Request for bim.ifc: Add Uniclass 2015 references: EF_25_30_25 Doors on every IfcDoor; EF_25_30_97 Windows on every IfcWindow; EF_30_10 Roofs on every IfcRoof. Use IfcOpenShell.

First a look at what the model holds.

```python
import ifcopenshell

model = ifcopenshell.open("bim.ifc")
print(model.schema)
print("classifications:", [c.Name for c in model.by_type("IfcClassification")])
for ifc_class in ("IfcDoor", "IfcRoof", "IfcStair", "IfcWall", "IfcWindow"):
    print(ifc_class, len(model.by_type(ifc_class)))
```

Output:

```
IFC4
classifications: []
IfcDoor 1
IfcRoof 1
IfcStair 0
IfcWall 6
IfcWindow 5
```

```python
import ifcopenshell
import ifcopenshell.api.classification

model = ifcopenshell.open("bim.ifc")

system = ifcopenshell.api.classification.add_classification(model, classification="Uniclass 2015")

codes = {
    "IfcDoor": ("EF_25_30_25", "Doors"),
    "IfcWindow": ("EF_25_30_97", "Windows"),
    "IfcRoof": ("EF_30_10", "Roofs"),
}
for ifc_class, (code, name) in codes.items():
    products = model.by_type(ifc_class)
    ifcopenshell.api.classification.add_reference(
        model, products=products, classification=system, identification=code, name=name
    )
    print(code, len(products))

model.write("bim_v2.ifc")
```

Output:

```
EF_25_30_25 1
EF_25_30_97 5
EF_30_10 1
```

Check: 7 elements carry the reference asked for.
